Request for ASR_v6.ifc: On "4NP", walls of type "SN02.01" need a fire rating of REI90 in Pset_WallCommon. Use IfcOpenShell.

First a look at what the model holds.

```python
import ifcopenshell
import ifcopenshell.util.element

model = ifcopenshell.open("ASR_v6.ifc")
print(model.schema)
storey = next(s for s in model.by_type("IfcBuildingStorey") if s.Name == "4NP")
walls = [e for e in ifcopenshell.util.element.get_decomposition(storey) if e.is_a("IfcWall")]
seen = {}
for e in walls:
    element_type = ifcopenshell.util.element.get_type(e)
    key = (element_type.Name if element_type != e and element_type else None, ifcopenshell.util.element.get_pset(e, "Pset_WallCommon", "FireRating"))
    seen[key] = seen.get(key, 0) + 1
for (name, value), count in sorted(seen.items(), key=str):
    print(count, "x", name, "|", value)
```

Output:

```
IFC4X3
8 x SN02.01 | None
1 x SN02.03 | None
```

```python
import ifcopenshell
import ifcopenshell.api.pset
import ifcopenshell.util.element

model = ifcopenshell.open("ASR_v6.ifc")

storey = next(s for s in model.by_type("IfcBuildingStorey") if s.Name == "4NP")
walls = [e for e in ifcopenshell.util.element.get_decomposition(storey) if e.is_a("IfcWall")]

count = 0
for e in walls:
    element_type = ifcopenshell.util.element.get_type(e)
    if element_type in (None, e) or element_type.Name != "SN02.01":
        continue
    # add_pset returns the element's existing set when there is one.
    pset = ifcopenshell.api.pset.add_pset(model, product=e, name="Pset_WallCommon")
    ifcopenshell.api.pset.edit_pset(model, pset=pset, properties={"FireRating": "REI90"})
    count += 1

print(count, "walls updated")

model.write("ASR_v6_v2.ifc")
```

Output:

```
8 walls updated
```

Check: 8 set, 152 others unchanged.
